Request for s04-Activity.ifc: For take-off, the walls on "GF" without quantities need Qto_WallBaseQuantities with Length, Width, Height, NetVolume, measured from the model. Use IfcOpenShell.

First a look at what the model holds.

```python
import ifcopenshell
import ifcopenshell.util.element
import ifcopenshell.util.unit

model = ifcopenshell.open("s04-Activity.ifc")
print(model.schema)
for unit_type in ("LENGTHUNIT", "AREAUNIT", "VOLUMEUNIT"):
    print(unit_type, ifcopenshell.util.unit.calculate_unit_scale(model, unit_type))
storey = next(s for s in model.by_type("IfcBuildingStorey") if s.Name == "GF")
walls = [e for e in ifcopenshell.util.element.get_decomposition(storey) if e.is_a("IfcWall")]
for e in sorted(walls, key=lambda e: e.id()):
    print(e.id(), e.is_a(), e.Name, list(ifcopenshell.util.element.get_psets(e, qtos_only=True)), sep=" | ")
```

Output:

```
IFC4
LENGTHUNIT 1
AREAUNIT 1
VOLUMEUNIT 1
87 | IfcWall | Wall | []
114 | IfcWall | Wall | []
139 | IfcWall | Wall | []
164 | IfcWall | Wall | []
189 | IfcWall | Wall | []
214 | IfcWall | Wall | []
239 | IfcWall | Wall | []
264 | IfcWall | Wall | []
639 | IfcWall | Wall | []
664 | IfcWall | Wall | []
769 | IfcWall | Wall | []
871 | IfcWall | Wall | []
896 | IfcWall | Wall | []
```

```python
import ifcopenshell
import ifcopenshell.api.pset
import ifcopenshell.geom
import ifcopenshell.util.element
import ifcopenshell.util.shape
import ifcopenshell.util.unit

model = ifcopenshell.open("s04-Activity.ifc")
unit_scale = ifcopenshell.util.unit.calculate_unit_scale(model)
volume_scale = ifcopenshell.util.unit.calculate_unit_scale(model, "VOLUMEUNIT")
settings = ifcopenshell.geom.settings()

storey = next(s for s in model.by_type("IfcBuildingStorey") if s.Name == "GF")
walls = [e for e in ifcopenshell.util.element.get_decomposition(storey) if e.is_a("IfcWall")]

for e in sorted(walls, key=lambda e: e.id()):
    if ifcopenshell.util.element.get_psets(e, qtos_only=True, should_inherit=False):
        continue
    # Geometry comes back in metres, in the element's own axes.
    shape = ifcopenshell.geom.create_shape(settings, e)
    values = {
        "Length": ifcopenshell.util.shape.get_x(shape.geometry) / unit_scale,
        "Width": ifcopenshell.util.shape.get_y(shape.geometry) / unit_scale,
        "Height": ifcopenshell.util.shape.get_z(shape.geometry) / unit_scale,
        "NetVolume": ifcopenshell.util.shape.get_volume(shape.geometry) / volume_scale,
    }
    qto = ifcopenshell.api.pset.add_qto(model, product=e, name="Qto_WallBaseQuantities")
    ifcopenshell.api.pset.edit_qto(model, qto=qto, properties=values)
    print(e.id(), {k: round(v, 3) for k, v in values.items()})

model.write("s04-Activity-out.ifc")
```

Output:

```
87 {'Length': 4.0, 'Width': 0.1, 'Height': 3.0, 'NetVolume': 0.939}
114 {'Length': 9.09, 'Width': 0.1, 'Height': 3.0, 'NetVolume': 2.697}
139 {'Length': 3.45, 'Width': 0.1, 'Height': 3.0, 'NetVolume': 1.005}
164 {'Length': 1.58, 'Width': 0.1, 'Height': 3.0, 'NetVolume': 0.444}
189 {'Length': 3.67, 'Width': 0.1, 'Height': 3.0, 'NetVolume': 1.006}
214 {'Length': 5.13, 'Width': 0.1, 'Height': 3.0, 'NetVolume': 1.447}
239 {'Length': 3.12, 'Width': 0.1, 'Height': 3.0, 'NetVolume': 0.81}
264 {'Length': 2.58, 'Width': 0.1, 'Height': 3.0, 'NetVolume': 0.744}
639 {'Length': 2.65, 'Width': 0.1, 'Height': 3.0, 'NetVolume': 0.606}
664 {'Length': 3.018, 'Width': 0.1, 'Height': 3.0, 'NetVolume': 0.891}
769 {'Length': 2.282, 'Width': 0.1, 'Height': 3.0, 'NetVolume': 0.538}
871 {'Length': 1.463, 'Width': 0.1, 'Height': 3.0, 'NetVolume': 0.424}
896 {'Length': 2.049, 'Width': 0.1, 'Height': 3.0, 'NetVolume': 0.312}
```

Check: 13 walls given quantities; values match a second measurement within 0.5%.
